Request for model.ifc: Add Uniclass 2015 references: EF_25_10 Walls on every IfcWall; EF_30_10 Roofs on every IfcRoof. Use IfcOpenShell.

First a look at what the model holds.

```python
import ifcopenshell

model = ifcopenshell.open("model.ifc")
print(model.schema)
print("classifications:", [c.Name for c in model.by_type("IfcClassification")])
for ifc_class in ("IfcDoor", "IfcRoof", "IfcStair", "IfcWall", "IfcWindow"):
    print(ifc_class, len(model.by_type(ifc_class)))
```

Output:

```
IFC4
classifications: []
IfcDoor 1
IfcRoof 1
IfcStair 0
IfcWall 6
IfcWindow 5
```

```python
import ifcopenshell
import ifcopenshell.api.classification

model = ifcopenshell.open("model.ifc")

system = ifcopenshell.api.classification.add_classification(model, classification="Uniclass 2015")

codes = {
    "IfcWall": ("EF_25_10", "Walls"),
    "IfcRoof": ("EF_30_10", "Roofs"),
}
for ifc_class, (code, name) in codes.items():
    products = model.by_type(ifc_class)
    ifcopenshell.api.classification.add_reference(
        model, products=products, classification=system, identification=code, name=name
    )
    print(code, len(products))

model.write("model_edited.ifc")
```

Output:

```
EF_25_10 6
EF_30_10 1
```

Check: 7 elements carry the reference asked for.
